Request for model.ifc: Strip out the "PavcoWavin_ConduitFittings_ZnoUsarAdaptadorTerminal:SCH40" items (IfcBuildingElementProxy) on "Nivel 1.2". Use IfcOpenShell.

First a look at what the model holds.

```python
import ifcopenshell
import ifcopenshell.util.element

model = ifcopenshell.open("model.ifc")
print(model.schema)
storey = next(s for s in model.by_type("IfcBuildingStorey") if s.Name == "Nivel 1.2")
proxies = [e for e in ifcopenshell.util.element.get_decomposition(storey) if e.is_a("IfcBuildingElementProxy")]
seen = {}
for e in proxies:
    element_type = ifcopenshell.util.element.get_type(e)
    name = element_type.Name if element_type not in (None, e) else None
    seen[name] = seen.get(name, 0) + 1
for name, count in sorted(seen.items(), key=str):
    print(count, "x", name)
```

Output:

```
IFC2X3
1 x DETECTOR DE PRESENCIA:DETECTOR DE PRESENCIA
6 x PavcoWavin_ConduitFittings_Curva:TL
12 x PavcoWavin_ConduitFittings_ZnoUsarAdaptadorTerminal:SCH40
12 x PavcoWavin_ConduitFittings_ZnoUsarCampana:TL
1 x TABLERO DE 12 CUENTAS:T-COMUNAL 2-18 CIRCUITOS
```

```python
import ifcopenshell
import ifcopenshell.api.root
import ifcopenshell.util.element

model = ifcopenshell.open("model.ifc")

storey = next(s for s in model.by_type("IfcBuildingStorey") if s.Name == "Nivel 1.2")
proxies = [e for e in ifcopenshell.util.element.get_decomposition(storey) if e.is_a("IfcBuildingElementProxy")]
targets = [e for e in proxies if (t := ifcopenshell.util.element.get_type(e)) not in (None, e) and t.Name == "PavcoWavin_ConduitFittings_ZnoUsarAdaptadorTerminal:SCH40"]

for e in targets:
    ifcopenshell.api.root.remove_product(model, product=e)
print(len(targets), "removed")

model.write("model_edited.ifc")
```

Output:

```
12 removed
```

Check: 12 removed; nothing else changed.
